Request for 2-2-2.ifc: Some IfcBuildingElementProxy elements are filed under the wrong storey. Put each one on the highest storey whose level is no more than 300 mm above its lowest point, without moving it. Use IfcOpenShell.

First a look at what the model holds.

```python
import ifcopenshell
import ifcopenshell.util.element
import ifcopenshell.util.placement

model = ifcopenshell.open("2-2-2.ifc")
print(model.schema)
for storey in model.by_type("IfcBuildingStorey"):
    level = ifcopenshell.util.placement.get_storey_elevation(storey)
    count = sum(e.is_a("IfcBuildingElementProxy") for e in ifcopenshell.util.element.get_contained(storey))
    print(storey.id(), storey.Name, round(level, 3), count, sep=" | ")
```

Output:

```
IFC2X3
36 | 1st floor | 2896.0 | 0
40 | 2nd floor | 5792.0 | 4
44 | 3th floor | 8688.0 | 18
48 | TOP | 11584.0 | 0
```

```python
import ifcopenshell
import ifcopenshell.api.spatial
import ifcopenshell.geom
import ifcopenshell.util.element
import ifcopenshell.util.placement
import ifcopenshell.util.shape
import ifcopenshell.util.unit

model = ifcopenshell.open("2-2-2.ifc")
unit_scale = ifcopenshell.util.unit.calculate_unit_scale(model)
settings = ifcopenshell.geom.settings()

levels = sorted(
    ((ifcopenshell.util.placement.get_storey_elevation(s) * unit_scale, s) for s in model.by_type("IfcBuildingStorey")),
    key=lambda pair: pair[0],
)

for e in model.by_type("IfcBuildingElementProxy"):
    current = e.ContainedInStructure[0].RelatingStructure if e.ContainedInStructure else None
    if current is None or not current.is_a("IfcBuildingStorey"):
        continue
    shape = ifcopenshell.geom.create_shape(settings, e)
    bottom = ifcopenshell.util.shape.get_shape_bottom_elevation(shape, shape.geometry)
    below = [s for level, s in levels if level <= bottom + 0.3]
    storey = below[-1] if below else levels[0][1]
    if storey != current:
        # assign_container keeps the world position.
        ifcopenshell.api.spatial.assign_container(model, products=[e], relating_structure=storey)
        print(e.id(), current.Name, "->", storey.Name)

model.write("2-2-2_rev.ifc")
```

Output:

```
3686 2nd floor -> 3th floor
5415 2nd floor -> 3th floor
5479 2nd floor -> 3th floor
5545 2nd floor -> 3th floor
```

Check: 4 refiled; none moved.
